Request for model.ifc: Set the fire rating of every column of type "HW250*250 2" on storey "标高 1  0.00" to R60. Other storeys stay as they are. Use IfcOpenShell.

First a look at what the model holds.

```python
import ifcopenshell
import ifcopenshell.util.element

model = ifcopenshell.open("model.ifc")
print(model.schema)
storey = next(s for s in model.by_type("IfcBuildingStorey") if s.Name == "标高 1  0.00")
columns = [e for e in ifcopenshell.util.element.get_decomposition(storey) if e.is_a("IfcColumn")]
seen = {}
for e in columns:
    element_type = ifcopenshell.util.element.get_type(e)
    key = (element_type.Name if element_type != e and element_type else None, ifcopenshell.util.element.get_pset(e, "Pset_ColumnCommon", "FireRating"))
    seen[key] = seen.get(key, 0) + 1
for (name, value), count in sorted(seen.items(), key=str):
    print(count, "x", name, "|", value)
```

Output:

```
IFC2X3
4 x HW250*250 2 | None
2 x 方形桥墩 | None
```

```python
import ifcopenshell
import ifcopenshell.api.pset
import ifcopenshell.util.element

model = ifcopenshell.open("model.ifc")

storey = next(s for s in model.by_type("IfcBuildingStorey") if s.Name == "标高 1  0.00")
columns = [e for e in ifcopenshell.util.element.get_decomposition(storey) if e.is_a("IfcColumn")]

count = 0
for e in columns:
    element_type = ifcopenshell.util.element.get_type(e)
    if element_type in (None, e) or element_type.Name != "HW250*250 2":
        continue
    # add_pset returns the element's existing set when there is one.
    pset = ifcopenshell.api.pset.add_pset(model, product=e, name="Pset_ColumnCommon")
    ifcopenshell.api.pset.edit_pset(model, pset=pset, properties={"FireRating": "R60"})
    count += 1

print(count, "columns updated")

model.write("model_rev.ifc")
```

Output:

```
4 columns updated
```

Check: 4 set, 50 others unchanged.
